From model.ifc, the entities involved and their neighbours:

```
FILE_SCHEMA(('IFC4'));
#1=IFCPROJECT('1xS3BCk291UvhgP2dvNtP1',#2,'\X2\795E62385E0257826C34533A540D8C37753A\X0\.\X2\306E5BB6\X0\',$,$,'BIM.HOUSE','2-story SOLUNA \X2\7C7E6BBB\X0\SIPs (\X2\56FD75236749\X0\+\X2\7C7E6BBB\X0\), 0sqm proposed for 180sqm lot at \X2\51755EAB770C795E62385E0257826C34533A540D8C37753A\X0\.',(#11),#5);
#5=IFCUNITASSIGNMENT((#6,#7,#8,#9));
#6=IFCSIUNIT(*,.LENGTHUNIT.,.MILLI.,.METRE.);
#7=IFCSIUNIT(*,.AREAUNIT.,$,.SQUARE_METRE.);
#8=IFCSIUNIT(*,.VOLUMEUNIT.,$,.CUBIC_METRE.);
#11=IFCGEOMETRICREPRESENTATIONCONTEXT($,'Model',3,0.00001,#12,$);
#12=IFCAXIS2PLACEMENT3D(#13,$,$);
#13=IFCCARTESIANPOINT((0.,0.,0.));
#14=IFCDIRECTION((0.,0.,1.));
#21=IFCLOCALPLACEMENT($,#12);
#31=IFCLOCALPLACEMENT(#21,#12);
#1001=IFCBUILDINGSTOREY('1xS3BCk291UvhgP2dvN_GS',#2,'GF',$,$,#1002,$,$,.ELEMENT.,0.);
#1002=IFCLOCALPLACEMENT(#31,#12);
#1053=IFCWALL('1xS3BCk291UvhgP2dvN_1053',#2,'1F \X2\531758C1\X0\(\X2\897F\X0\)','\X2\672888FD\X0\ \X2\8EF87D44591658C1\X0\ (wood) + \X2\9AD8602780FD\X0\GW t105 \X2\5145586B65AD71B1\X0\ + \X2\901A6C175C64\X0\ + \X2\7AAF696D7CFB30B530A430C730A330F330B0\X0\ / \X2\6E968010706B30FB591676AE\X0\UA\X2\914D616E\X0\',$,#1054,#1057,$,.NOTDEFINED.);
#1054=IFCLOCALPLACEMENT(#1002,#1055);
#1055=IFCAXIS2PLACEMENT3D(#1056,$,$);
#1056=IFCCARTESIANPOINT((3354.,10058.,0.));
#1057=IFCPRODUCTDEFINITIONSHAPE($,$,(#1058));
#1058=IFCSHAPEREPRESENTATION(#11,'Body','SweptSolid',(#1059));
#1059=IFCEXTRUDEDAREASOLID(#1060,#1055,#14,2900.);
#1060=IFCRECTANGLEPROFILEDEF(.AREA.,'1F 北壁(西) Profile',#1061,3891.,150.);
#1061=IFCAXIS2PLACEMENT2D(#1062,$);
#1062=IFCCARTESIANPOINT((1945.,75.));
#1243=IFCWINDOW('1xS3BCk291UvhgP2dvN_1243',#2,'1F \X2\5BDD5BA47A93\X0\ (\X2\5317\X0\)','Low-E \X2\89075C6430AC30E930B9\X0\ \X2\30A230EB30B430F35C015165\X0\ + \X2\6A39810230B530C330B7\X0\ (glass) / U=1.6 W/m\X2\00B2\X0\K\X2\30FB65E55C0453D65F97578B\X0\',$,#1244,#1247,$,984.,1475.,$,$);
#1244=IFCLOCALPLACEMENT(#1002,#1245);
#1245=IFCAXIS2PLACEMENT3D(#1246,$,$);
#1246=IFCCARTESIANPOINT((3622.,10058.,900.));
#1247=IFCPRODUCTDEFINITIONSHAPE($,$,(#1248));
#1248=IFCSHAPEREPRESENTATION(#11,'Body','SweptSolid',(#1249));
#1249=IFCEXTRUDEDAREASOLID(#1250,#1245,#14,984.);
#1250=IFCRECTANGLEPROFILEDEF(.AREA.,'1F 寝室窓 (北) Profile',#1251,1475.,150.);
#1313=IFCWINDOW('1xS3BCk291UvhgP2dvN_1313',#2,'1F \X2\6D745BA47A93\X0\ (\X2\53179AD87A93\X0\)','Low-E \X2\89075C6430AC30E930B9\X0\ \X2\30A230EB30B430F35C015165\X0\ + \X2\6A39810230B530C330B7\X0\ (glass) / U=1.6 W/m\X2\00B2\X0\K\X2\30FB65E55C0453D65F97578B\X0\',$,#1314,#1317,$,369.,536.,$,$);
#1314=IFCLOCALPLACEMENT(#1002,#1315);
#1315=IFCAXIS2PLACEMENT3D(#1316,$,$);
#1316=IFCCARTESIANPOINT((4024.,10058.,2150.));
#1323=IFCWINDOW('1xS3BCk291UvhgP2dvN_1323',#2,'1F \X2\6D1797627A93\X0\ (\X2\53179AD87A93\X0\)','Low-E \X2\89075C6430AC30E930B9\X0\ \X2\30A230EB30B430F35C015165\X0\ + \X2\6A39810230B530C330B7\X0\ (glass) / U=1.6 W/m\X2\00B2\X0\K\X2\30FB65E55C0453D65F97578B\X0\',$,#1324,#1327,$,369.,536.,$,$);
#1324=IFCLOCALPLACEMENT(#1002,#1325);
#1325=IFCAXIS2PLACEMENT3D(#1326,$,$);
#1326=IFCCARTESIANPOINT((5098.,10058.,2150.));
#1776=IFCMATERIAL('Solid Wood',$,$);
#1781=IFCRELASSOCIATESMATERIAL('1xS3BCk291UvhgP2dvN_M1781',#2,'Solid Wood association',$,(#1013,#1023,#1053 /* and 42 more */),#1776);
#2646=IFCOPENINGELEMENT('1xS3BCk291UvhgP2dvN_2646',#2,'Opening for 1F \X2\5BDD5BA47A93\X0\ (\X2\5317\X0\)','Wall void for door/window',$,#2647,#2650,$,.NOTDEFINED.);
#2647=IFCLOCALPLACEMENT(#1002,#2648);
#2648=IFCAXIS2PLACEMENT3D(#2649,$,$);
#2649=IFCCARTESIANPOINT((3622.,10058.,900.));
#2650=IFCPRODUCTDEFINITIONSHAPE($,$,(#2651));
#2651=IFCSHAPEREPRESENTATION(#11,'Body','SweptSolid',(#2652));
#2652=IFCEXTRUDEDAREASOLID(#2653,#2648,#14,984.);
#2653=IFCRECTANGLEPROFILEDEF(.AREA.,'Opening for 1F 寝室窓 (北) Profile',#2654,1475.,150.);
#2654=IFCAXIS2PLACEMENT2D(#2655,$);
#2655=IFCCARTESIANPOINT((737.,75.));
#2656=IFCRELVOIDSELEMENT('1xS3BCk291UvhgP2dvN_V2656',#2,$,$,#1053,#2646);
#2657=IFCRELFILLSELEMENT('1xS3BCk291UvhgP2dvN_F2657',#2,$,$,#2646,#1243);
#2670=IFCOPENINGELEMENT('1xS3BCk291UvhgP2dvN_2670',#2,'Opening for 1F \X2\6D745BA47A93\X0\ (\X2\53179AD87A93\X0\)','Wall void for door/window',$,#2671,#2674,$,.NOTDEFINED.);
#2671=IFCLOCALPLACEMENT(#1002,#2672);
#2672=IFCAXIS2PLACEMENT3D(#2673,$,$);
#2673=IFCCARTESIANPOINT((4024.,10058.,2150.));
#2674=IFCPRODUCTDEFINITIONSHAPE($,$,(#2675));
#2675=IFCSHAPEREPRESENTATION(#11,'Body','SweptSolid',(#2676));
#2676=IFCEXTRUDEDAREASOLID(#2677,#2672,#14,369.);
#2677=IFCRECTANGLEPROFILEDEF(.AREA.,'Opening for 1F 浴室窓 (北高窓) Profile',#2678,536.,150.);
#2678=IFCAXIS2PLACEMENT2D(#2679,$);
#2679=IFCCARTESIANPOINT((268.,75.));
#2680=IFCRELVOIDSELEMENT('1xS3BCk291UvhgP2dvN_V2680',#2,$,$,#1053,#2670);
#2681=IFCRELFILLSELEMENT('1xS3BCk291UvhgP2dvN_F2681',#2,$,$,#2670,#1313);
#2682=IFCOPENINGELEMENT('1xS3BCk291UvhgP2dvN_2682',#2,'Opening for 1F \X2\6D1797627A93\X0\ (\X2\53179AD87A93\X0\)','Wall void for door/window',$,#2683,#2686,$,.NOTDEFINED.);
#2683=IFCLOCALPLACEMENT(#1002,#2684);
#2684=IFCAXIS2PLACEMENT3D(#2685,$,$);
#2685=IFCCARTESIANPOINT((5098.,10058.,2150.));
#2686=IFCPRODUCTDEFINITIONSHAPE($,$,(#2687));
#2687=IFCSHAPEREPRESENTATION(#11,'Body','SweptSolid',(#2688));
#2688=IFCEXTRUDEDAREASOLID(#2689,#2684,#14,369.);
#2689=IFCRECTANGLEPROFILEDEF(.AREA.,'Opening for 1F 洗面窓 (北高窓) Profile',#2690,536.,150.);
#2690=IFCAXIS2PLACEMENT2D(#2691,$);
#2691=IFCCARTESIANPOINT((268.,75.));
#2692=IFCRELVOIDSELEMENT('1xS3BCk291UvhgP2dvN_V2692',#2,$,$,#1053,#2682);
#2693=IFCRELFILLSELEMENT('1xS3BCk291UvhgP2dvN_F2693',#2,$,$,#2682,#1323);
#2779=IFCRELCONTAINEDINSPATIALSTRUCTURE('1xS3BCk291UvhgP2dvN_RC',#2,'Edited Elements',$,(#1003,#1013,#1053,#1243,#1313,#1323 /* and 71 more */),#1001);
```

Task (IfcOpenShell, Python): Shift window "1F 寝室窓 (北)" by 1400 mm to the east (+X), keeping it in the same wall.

```python
import ifcopenshell
import ifcopenshell.api.geometry
import ifcopenshell.util.placement
import ifcopenshell.util.unit

model = ifcopenshell.open("model.ifc")
unit_scale = ifcopenshell.util.unit.calculate_unit_scale(model)

window = model.by_guid("1xS3BCk291UvhgP2dvN_1243")
opening = window.FillsVoids[0].RelatingOpeningElement
wall = opening.VoidsElements[0].RelatingBuildingElement

wall_matrix = ifcopenshell.util.placement.get_local_placement(wall.ObjectPlacement)
shift = wall_matrix[:3, 0] * 1.4 / unit_scale
before = ifcopenshell.util.placement.get_local_placement(window.ObjectPlacement)[:3, 3].copy()

# The window is not placed relative to its opening, so move both.
for product in (opening, window):
    matrix = ifcopenshell.util.placement.get_local_placement(product.ObjectPlacement)
    matrix[:3, 3] += shift
    ifcopenshell.api.geometry.edit_object_placement(model, product=product, matrix=matrix, is_si=False)

after = ifcopenshell.util.placement.get_local_placement(window.ObjectPlacement)[:3, 3]
print("window moved by", (after - before).round(3) + 0.0)

model.write("model_updated.ifc")
```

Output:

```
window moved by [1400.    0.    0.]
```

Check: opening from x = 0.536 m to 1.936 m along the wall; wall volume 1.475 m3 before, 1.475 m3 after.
